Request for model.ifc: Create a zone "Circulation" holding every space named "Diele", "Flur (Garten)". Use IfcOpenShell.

First a look at what the model holds.

```python
import ifcopenshell

model = ifcopenshell.open("model.ifc")
print(model.schema)
seen = {}
for space in model.by_type("IfcSpace"):
    seen[space.LongName] = seen.get(space.LongName, 0) + 1
for name, count in sorted(seen.items(), key=str):
    print(count, "x", name)
print("zones:", [z.Name for z in model.by_type("IfcZone")][:20])
```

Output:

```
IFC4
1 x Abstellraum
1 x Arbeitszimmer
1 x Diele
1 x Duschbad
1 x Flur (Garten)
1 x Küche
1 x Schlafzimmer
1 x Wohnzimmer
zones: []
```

```python
import ifcopenshell
import ifcopenshell.api.group
import ifcopenshell.api.root

model = ifcopenshell.open("model.ifc")

names = {"Diele", "Flur (Garten)"}
spaces = [s for s in model.by_type("IfcSpace") if s.LongName in names]

zone = ifcopenshell.api.root.create_entity(model, ifc_class="IfcZone", name="Circulation")
ifcopenshell.api.group.assign_group(model, products=spaces, group=zone)
print(len(spaces), "spaces in", zone.Name)

model.write("model_rev.ifc")
```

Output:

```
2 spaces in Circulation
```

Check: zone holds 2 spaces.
